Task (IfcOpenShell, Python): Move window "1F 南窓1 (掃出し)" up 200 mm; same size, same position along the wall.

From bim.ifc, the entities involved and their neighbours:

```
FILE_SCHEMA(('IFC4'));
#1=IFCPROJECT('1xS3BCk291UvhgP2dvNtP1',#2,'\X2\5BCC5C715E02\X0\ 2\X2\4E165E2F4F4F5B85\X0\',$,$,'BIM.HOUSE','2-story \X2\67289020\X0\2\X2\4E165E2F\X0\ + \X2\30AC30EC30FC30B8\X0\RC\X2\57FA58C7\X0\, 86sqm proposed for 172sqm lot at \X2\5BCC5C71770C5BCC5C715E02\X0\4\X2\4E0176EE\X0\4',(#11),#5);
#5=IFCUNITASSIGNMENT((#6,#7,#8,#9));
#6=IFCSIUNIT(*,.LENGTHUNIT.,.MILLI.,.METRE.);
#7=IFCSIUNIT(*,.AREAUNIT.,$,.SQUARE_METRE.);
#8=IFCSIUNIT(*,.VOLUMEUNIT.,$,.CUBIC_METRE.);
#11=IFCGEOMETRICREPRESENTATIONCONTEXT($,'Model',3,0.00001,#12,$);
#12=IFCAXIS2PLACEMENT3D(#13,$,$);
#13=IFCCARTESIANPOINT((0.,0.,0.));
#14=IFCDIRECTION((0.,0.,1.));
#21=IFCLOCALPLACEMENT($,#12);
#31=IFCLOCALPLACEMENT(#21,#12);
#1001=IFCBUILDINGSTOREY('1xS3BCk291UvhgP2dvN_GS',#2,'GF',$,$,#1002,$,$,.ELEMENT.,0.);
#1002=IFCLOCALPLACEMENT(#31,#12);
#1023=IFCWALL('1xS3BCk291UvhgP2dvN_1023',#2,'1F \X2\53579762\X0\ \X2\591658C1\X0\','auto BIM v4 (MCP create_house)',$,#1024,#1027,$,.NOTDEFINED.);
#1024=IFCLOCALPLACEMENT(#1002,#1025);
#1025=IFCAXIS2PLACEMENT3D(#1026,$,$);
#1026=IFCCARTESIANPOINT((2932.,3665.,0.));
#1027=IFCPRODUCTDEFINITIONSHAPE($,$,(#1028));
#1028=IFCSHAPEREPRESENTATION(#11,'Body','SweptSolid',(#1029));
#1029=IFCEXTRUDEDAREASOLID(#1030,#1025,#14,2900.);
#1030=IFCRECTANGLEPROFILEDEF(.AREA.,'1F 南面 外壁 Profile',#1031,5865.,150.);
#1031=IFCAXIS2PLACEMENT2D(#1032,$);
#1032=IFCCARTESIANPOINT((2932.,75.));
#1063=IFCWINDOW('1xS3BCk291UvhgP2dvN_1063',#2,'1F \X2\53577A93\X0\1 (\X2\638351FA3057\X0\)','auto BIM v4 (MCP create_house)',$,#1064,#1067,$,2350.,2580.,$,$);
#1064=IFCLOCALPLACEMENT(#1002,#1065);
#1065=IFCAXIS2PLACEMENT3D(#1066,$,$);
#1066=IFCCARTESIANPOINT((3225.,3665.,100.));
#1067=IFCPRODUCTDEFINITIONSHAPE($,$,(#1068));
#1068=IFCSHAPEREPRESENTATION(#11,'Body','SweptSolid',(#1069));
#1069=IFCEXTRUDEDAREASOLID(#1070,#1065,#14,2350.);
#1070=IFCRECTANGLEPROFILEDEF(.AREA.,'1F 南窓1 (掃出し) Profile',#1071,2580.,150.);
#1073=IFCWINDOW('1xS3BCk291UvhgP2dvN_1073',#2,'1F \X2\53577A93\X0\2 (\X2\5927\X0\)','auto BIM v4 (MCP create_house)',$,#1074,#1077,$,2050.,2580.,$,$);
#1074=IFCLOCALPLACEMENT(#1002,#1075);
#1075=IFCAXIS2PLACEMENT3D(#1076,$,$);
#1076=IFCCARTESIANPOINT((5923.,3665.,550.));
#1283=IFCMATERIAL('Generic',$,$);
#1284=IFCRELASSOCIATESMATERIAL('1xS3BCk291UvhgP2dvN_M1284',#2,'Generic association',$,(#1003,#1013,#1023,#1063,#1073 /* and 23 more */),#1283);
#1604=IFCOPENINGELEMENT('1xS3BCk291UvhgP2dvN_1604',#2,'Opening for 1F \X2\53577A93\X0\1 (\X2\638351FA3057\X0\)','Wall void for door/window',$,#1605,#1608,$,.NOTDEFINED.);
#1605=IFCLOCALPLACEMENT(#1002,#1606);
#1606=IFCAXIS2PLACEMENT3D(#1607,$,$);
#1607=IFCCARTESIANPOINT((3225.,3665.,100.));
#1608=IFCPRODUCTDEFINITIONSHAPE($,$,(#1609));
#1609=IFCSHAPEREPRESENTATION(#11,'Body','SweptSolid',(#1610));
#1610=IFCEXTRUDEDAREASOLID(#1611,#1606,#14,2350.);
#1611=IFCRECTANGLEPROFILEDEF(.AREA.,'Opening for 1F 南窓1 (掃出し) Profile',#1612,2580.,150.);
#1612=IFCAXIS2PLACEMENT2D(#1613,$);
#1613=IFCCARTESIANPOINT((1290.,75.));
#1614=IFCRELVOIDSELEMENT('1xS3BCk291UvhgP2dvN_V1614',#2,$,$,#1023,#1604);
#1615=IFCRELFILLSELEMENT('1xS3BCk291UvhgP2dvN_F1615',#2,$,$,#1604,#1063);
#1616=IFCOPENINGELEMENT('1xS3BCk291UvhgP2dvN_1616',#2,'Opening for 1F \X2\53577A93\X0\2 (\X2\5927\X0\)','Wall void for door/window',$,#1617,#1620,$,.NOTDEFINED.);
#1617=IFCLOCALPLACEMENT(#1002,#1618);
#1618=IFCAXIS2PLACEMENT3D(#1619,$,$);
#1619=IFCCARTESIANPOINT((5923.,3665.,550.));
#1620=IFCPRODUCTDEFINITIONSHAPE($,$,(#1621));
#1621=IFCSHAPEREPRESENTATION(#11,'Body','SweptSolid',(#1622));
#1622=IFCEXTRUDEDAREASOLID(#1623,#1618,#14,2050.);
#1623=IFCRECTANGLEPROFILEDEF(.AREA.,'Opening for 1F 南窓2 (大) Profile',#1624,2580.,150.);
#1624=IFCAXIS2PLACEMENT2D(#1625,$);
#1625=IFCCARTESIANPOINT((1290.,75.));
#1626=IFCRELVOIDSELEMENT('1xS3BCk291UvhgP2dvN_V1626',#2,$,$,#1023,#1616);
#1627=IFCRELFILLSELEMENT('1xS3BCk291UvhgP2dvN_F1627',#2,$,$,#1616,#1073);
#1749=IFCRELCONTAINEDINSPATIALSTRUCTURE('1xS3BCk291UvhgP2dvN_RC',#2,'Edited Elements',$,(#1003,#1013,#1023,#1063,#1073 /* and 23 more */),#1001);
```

```python
import numpy as np
import ifcopenshell
import ifcopenshell.api.geometry
import ifcopenshell.util.placement
import ifcopenshell.util.unit

model = ifcopenshell.open("bim.ifc")
unit_scale = ifcopenshell.util.unit.calculate_unit_scale(model)

window = model.by_guid("1xS3BCk291UvhgP2dvN_1063")
opening = window.FillsVoids[0].RelatingOpeningElement
dz = 200.0

shift = np.array([0.0, 0.0, dz])
# The window is not placed relative to its opening, so move both.
for product in (opening, window):
    matrix = ifcopenshell.util.placement.get_local_placement(product.ObjectPlacement)
    matrix[:3, 3] += shift
    ifcopenshell.api.geometry.edit_object_placement(model, product=product, matrix=matrix, is_si=False)

print(f"moved by {dz * unit_scale:+.3f} m")

model.write("bim_v2.ifc")
```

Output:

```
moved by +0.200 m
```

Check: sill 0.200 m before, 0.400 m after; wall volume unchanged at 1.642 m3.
